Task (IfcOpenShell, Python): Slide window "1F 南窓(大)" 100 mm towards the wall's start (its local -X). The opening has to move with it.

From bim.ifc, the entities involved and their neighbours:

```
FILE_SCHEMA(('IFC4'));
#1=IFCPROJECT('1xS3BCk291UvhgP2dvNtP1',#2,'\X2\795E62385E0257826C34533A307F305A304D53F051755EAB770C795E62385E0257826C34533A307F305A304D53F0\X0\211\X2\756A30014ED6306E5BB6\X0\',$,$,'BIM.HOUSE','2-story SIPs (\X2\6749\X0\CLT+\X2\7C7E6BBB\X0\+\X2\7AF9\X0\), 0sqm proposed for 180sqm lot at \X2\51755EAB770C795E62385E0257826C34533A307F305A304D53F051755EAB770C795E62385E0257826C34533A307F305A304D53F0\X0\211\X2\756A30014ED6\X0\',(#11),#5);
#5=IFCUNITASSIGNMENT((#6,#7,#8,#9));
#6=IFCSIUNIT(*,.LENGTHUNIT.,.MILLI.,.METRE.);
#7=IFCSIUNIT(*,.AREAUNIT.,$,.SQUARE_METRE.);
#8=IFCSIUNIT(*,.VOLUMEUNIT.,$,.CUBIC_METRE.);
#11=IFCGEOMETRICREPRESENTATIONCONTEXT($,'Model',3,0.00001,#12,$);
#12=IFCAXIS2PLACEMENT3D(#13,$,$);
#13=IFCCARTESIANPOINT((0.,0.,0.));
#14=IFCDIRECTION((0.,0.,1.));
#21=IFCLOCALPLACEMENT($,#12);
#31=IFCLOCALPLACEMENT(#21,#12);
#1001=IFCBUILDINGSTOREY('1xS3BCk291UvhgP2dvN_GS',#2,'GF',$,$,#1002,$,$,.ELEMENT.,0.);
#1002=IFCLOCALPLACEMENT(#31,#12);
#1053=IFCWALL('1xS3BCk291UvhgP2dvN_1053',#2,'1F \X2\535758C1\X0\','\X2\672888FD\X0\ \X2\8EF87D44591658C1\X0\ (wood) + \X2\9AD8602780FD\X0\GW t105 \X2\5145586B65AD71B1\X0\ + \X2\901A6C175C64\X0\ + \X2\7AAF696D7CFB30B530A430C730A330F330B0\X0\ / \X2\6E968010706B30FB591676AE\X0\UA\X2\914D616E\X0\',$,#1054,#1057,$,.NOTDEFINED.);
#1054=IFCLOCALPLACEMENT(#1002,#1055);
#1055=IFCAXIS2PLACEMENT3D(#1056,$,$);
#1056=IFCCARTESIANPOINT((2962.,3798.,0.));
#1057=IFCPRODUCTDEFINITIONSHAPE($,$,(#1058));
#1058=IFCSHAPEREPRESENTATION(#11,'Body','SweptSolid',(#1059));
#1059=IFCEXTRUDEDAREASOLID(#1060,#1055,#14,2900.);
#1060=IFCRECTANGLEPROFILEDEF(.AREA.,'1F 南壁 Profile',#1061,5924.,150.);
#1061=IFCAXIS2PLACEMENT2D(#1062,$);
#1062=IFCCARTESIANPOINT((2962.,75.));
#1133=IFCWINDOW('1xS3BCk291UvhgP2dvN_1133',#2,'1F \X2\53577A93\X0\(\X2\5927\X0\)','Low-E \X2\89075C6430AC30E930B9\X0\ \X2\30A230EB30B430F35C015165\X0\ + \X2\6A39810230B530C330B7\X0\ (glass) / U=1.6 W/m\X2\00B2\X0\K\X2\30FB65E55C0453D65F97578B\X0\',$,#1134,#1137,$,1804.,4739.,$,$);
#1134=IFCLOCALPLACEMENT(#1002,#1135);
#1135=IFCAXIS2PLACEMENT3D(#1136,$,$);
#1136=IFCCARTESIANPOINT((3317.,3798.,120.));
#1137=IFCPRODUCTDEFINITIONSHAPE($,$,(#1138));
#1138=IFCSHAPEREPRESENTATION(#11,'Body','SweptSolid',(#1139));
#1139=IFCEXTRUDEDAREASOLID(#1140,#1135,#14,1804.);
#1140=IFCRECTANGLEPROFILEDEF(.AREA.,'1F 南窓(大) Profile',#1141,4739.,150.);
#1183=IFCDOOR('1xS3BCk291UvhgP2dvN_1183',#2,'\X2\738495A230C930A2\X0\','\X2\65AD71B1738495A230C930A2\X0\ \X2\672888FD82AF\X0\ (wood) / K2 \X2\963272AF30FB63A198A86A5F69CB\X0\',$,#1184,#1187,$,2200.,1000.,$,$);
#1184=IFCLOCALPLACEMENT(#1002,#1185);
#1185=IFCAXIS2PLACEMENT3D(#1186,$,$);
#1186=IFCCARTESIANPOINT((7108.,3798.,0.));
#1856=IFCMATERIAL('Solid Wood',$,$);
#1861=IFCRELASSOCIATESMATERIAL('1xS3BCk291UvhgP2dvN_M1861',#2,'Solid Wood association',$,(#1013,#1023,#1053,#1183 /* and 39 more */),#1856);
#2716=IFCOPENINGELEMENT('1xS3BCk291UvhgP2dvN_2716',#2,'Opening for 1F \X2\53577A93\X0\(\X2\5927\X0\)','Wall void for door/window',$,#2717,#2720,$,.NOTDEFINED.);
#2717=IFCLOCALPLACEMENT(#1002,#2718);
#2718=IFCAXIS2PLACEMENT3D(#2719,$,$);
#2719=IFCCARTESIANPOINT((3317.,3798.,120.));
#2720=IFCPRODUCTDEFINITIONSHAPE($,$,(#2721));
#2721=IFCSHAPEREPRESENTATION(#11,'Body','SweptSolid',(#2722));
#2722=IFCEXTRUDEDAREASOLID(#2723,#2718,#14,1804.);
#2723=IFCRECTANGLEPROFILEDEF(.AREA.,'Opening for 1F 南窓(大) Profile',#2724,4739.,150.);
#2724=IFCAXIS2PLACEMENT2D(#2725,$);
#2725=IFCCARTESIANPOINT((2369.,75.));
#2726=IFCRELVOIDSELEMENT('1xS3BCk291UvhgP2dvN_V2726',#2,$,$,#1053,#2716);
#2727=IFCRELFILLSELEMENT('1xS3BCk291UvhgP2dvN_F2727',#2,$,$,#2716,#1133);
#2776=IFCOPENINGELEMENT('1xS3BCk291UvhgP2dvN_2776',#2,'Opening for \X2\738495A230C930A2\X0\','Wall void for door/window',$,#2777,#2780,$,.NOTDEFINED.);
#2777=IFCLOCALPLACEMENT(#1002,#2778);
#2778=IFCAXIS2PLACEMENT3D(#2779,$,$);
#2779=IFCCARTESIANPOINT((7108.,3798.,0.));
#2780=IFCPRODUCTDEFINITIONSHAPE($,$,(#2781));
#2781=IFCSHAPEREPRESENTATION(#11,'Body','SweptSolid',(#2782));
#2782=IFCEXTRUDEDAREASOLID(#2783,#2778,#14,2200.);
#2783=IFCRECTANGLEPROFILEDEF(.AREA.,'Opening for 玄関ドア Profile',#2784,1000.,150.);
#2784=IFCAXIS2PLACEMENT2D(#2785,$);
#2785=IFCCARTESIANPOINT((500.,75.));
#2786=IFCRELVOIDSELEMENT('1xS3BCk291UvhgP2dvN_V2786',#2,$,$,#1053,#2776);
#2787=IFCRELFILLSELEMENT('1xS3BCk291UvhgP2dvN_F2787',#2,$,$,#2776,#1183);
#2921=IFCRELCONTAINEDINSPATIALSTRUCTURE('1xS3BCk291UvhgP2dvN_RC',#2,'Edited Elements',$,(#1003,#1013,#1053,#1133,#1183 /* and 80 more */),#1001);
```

```python
import ifcopenshell
import ifcopenshell.api.geometry
import ifcopenshell.util.placement

model = ifcopenshell.open("bim.ifc")

window = model.by_guid("1xS3BCk291UvhgP2dvN_1133")
opening = window.FillsVoids[0].RelatingOpeningElement
wall = opening.VoidsElements[0].RelatingBuildingElement

wall_matrix = ifcopenshell.util.placement.get_local_placement(wall.ObjectPlacement)
shift = wall_matrix[:3, 0] * -100.0
before = ifcopenshell.util.placement.get_local_placement(window.ObjectPlacement)[:3, 3].copy()

# The window is not placed relative to its opening, so move both.
for product in (opening, window):
    matrix = ifcopenshell.util.placement.get_local_placement(product.ObjectPlacement)
    matrix[:3, 3] += shift
    ifcopenshell.api.geometry.edit_object_placement(model, product=product, matrix=matrix, is_si=False)

after = ifcopenshell.util.placement.get_local_placement(window.ObjectPlacement)[:3, 3]
print("window moved by", (after - before).round(3) + 0.0)

model.write("bim_updated.ifc")
```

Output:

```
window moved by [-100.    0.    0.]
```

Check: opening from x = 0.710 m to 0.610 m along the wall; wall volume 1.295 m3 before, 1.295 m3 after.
